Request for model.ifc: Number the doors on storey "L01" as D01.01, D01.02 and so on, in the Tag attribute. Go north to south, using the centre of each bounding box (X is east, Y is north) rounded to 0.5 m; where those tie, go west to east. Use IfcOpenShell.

First a look at what the model holds.

```python
import ifcopenshell
import ifcopenshell.util.element
import ifcopenshell.util.placement

model = ifcopenshell.open("model.ifc")
print(model.schema)
storey = next(s for s in model.by_type("IfcBuildingStorey") if s.Name == "L01")
doors = [e for e in ifcopenshell.util.element.get_decomposition(storey) if e.is_a("IfcDoor")]
for e in sorted(doors, key=lambda e: e.id()):
    origin = ifcopenshell.util.placement.get_local_placement(e.ObjectPlacement)[:3, 3]
    print(e.id(), e.Tag, e.Name, origin.round(2) + 0.0, sep=" | ")
```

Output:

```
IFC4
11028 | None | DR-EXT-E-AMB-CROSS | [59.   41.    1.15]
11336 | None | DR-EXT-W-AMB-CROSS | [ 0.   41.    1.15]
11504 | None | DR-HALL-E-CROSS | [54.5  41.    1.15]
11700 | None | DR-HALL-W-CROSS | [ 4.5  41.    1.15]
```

```python
import ifcopenshell
import ifcopenshell.geom
import ifcopenshell.util.element
import ifcopenshell.util.shape

model = ifcopenshell.open("model.ifc")
settings = ifcopenshell.geom.settings()
settings.set("use-world-coords", True)


def centre(element):
    shape = ifcopenshell.geom.create_shape(settings, element)
    return ifcopenshell.util.shape.get_bbox_centroid(shape.geometry)


storey = next(s for s in model.by_type("IfcBuildingStorey") if s.Name == "L01")
doors = [e for e in ifcopenshell.util.element.get_decomposition(storey) if e.is_a("IfcDoor")]

# Insertion points can sit at a corner or the storey origin, so sort by the geometry (in metres).
centres = {e: centre(e) for e in doors}
doors.sort(key=lambda e: (-round(centres[e][1] / 0.5), centres[e][0]))

for i, e in enumerate(doors, start=1):
    number = f"D01.{i:02d}"
    e.Tag = number
    print(e.id(), number)

model.write("model_edited.ifc")
```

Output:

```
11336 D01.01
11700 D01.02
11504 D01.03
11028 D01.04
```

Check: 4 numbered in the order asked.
